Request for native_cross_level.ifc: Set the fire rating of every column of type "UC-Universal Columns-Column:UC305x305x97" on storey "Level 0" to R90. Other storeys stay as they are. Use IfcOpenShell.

First a look at what the model holds.

```python
import ifcopenshell
import ifcopenshell.util.element

model = ifcopenshell.open("native_cross_level.ifc")
print(model.schema)
storey = next(s for s in model.by_type("IfcBuildingStorey") if s.Name == "Level 0")
columns = [e for e in ifcopenshell.util.element.get_decomposition(storey) if e.is_a("IfcColumn")]
seen = {}
for e in columns:
    element_type = ifcopenshell.util.element.get_type(e)
    key = (element_type.Name if element_type != e and element_type else None, ifcopenshell.util.element.get_pset(e, "Pset_ColumnCommon", "FireRating"))
    seen[key] = seen.get(key, 0) + 1
for (name, value), count in sorted(seen.items(), key=str):
    print(count, "x", name, "|", value)
```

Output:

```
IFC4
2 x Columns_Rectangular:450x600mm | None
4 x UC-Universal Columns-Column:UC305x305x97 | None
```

```python
import ifcopenshell
import ifcopenshell.api.pset
import ifcopenshell.util.element

model = ifcopenshell.open("native_cross_level.ifc")

storey = next(s for s in model.by_type("IfcBuildingStorey") if s.Name == "Level 0")
columns = [e for e in ifcopenshell.util.element.get_decomposition(storey) if e.is_a("IfcColumn")]

count = 0
for e in columns:
    element_type = ifcopenshell.util.element.get_type(e)
    if element_type in (None, e) or element_type.Name != "UC-Universal Columns-Column:UC305x305x97":
        continue
    # add_pset returns the element's existing set when there is one.
    pset = ifcopenshell.api.pset.add_pset(model, product=e, name="Pset_ColumnCommon")
    ifcopenshell.api.pset.edit_pset(model, pset=pset, properties={"FireRating": "R90"})
    count += 1

print(count, "columns updated")

model.write("native_cross_level_v2.ifc")
```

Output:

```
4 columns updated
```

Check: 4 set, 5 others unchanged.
